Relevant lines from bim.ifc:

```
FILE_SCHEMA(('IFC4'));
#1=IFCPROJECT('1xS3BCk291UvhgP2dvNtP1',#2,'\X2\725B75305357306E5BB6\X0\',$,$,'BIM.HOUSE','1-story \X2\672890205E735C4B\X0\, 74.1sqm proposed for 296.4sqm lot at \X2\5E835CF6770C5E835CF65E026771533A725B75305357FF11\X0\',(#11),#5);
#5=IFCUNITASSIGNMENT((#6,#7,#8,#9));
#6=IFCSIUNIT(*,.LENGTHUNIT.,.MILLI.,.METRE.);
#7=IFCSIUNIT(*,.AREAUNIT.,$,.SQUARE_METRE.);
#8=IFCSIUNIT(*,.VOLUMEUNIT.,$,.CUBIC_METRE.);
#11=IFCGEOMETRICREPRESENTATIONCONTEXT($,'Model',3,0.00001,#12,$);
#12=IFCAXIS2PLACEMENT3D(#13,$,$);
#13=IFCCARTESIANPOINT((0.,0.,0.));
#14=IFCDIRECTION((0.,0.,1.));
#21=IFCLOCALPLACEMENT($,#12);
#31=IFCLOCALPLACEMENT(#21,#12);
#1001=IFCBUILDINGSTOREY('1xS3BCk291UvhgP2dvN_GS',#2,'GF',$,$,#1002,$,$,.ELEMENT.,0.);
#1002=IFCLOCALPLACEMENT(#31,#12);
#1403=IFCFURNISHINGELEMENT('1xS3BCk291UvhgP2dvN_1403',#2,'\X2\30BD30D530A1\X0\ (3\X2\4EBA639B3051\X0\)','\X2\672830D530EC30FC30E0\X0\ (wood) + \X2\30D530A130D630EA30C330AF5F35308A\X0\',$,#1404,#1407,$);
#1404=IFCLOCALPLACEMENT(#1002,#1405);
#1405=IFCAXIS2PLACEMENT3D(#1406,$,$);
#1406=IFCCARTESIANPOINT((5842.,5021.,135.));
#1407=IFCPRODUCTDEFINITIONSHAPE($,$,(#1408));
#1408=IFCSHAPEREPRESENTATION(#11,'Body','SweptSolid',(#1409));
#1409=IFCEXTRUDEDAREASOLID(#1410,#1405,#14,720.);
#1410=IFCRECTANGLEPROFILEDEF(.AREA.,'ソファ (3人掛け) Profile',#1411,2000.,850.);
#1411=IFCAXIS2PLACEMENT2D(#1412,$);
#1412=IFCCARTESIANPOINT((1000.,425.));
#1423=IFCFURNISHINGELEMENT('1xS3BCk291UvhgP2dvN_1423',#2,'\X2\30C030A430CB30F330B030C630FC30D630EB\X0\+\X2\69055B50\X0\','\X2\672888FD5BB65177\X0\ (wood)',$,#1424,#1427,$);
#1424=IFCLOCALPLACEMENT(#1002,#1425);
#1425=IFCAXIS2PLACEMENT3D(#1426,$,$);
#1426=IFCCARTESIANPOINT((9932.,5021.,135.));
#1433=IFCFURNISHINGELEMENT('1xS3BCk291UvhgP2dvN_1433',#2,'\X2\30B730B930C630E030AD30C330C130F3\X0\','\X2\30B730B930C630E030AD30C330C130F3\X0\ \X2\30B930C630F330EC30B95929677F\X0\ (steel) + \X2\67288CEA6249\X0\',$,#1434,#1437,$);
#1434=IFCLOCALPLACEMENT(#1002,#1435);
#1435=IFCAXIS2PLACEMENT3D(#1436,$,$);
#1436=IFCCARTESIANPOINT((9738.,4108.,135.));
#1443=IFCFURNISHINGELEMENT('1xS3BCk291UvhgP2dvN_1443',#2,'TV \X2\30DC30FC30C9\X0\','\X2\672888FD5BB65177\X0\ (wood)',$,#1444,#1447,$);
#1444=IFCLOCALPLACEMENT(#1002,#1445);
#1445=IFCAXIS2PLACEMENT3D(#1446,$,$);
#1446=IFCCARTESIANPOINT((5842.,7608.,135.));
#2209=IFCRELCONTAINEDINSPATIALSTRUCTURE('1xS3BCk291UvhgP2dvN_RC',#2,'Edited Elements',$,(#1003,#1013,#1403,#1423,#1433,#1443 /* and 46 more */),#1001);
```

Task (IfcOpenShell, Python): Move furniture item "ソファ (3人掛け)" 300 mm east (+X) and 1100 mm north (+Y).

```python
import ifcopenshell
import ifcopenshell.api.geometry
import ifcopenshell.util.placement

model = ifcopenshell.open("bim.ifc")

item = model.by_id(1403)
matrix = ifcopenshell.util.placement.get_local_placement(item.ObjectPlacement)
matrix[0, 3] += 300.0
matrix[1, 3] += 1100.0
ifcopenshell.api.geometry.edit_object_placement(model, product=item, matrix=matrix, is_si=False)

print(ifcopenshell.util.placement.get_local_placement(item.ObjectPlacement).round(3) + 0.0)

model.write("bim-out.ifc")
```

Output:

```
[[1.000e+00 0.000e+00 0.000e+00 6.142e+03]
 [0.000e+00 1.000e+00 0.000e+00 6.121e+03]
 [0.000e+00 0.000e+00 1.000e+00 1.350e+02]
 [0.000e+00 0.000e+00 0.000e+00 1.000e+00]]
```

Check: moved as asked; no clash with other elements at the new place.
